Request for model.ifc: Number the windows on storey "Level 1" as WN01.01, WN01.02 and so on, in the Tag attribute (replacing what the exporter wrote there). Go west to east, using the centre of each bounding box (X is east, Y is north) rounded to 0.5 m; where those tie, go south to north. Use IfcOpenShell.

First a look at what the model holds.

```python
import ifcopenshell
import ifcopenshell.util.element
import ifcopenshell.util.placement

model = ifcopenshell.open("model.ifc")
print(model.schema)
storey = next(s for s in model.by_type("IfcBuildingStorey") if s.Name == "Level 1")
windows = [e for e in ifcopenshell.util.element.get_decomposition(storey) if e.is_a("IfcWindow")]
for e in sorted(windows, key=lambda e: e.id()):
    origin = ifcopenshell.util.placement.get_local_placement(e.ObjectPlacement)[:3, 3]
    print(e.id(), e.Tag, e.Name, origin.round(2) + 0.0, sep=" | ")
```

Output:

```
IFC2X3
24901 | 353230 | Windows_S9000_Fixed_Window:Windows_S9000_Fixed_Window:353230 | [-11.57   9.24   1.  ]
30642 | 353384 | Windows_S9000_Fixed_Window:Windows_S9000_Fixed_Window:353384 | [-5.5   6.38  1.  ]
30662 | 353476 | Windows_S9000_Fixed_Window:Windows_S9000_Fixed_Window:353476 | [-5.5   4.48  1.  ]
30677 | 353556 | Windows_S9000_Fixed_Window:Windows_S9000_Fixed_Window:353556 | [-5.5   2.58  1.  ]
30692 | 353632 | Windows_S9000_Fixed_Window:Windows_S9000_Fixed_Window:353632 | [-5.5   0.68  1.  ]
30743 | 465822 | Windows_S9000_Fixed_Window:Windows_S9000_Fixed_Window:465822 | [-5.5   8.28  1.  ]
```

```python
import ifcopenshell
import ifcopenshell.geom
import ifcopenshell.util.element
import ifcopenshell.util.shape

model = ifcopenshell.open("model.ifc")
settings = ifcopenshell.geom.settings()
settings.set("use-world-coords", True)


def centre(element):
    shape = ifcopenshell.geom.create_shape(settings, element)
    return ifcopenshell.util.shape.get_bbox_centroid(shape.geometry)


storey = next(s for s in model.by_type("IfcBuildingStorey") if s.Name == "Level 1")
windows = [e for e in ifcopenshell.util.element.get_decomposition(storey) if e.is_a("IfcWindow")]

# Insertion points can sit at a corner or the storey origin, so sort by the geometry (in metres).
centres = {e: centre(e) for e in windows}
windows.sort(key=lambda e: (round(centres[e][0] / 0.5), centres[e][1]))

for i, e in enumerate(windows, start=1):
    number = f"WN01.{i:02d}"
    e.Tag = number
    print(e.id(), number)

model.write("model_updated.ifc")
```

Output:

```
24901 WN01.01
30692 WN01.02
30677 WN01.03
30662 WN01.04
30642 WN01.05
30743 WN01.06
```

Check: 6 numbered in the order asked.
